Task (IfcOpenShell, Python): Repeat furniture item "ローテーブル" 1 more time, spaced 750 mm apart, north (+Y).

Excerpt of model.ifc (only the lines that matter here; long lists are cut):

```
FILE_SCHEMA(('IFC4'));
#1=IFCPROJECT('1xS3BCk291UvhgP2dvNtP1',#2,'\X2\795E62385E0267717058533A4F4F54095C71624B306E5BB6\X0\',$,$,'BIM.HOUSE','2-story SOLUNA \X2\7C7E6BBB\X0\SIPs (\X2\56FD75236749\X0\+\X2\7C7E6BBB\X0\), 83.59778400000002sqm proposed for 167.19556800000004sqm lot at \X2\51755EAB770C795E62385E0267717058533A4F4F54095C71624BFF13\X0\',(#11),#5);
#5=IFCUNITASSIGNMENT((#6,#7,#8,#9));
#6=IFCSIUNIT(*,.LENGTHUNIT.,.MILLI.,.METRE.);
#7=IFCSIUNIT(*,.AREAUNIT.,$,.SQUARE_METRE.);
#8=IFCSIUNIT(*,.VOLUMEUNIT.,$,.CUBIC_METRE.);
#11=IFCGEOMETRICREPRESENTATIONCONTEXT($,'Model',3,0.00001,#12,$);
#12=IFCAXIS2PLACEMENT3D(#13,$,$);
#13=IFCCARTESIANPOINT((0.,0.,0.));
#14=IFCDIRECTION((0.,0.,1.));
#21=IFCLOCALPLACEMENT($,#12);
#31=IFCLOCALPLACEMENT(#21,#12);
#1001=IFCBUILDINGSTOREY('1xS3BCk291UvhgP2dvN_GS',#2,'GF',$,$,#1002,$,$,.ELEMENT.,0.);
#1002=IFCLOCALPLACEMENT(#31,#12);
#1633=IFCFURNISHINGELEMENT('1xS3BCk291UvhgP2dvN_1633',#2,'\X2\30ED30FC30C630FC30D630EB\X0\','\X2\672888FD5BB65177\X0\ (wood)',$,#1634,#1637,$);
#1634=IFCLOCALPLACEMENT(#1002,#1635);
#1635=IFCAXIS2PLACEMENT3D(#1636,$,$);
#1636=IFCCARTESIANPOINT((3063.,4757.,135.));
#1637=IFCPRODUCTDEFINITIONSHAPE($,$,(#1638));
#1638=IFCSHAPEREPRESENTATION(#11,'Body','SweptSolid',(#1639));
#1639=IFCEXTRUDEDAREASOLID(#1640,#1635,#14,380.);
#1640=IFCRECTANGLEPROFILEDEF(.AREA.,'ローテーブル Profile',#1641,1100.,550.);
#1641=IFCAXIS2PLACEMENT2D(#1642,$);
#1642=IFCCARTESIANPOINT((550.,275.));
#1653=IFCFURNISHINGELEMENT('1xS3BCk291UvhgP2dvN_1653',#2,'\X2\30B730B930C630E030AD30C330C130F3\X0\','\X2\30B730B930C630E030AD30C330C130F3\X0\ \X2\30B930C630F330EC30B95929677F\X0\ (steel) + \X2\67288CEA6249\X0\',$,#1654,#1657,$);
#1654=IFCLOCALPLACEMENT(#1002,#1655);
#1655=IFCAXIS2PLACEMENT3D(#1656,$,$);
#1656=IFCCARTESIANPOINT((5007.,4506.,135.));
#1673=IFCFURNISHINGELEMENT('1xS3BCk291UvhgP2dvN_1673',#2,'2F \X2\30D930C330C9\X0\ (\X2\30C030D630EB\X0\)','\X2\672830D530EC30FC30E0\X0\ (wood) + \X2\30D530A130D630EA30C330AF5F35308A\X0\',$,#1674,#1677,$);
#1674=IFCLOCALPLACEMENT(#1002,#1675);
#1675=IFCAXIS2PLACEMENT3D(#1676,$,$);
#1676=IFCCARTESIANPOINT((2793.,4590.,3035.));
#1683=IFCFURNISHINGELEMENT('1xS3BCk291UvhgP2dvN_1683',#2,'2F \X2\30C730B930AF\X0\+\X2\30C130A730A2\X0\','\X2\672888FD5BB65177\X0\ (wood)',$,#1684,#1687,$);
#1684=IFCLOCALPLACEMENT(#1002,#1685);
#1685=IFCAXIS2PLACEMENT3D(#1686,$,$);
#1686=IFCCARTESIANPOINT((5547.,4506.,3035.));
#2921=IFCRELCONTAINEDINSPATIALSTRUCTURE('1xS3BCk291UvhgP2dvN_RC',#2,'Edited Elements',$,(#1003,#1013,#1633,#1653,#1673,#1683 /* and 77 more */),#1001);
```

```python
import numpy as np
import ifcopenshell
import ifcopenshell.api.geometry
import ifcopenshell.api.root
import ifcopenshell.util.element
import ifcopenshell.util.placement
import ifcopenshell.util.unit

model = ifcopenshell.open("model.ifc")
unit_scale = ifcopenshell.util.unit.calculate_unit_scale(model)


def reuse_history(source, copy):
    """copy_class also copies each property set's owner history, people and application; keep the originals."""
    for rel in copy.IsDefinedBy:
        if rel.is_a("IfcRelDefinesByProperties") and (history := rel.RelatingPropertyDefinition.OwnerHistory):
            rel.RelatingPropertyDefinition.OwnerHistory = source.OwnerHistory
            ifcopenshell.util.element.remove_deep2(model, history)


source = model.by_guid("1xS3BCk291UvhgP2dvN_1633")
base = ifcopenshell.util.placement.get_local_placement(source.ObjectPlacement)
step = np.array([0.0, 1.0, 0.0]) * 0.75 / unit_scale

for i in range(1, 2):
    copy = ifcopenshell.api.root.copy_class(model, product=source)
    copy.Representation = ifcopenshell.util.element.copy_deep(
        model, source.Representation, exclude=["IfcGeometricRepresentationContext", "IfcRepresentationMap"]
    )
    reuse_history(source, copy)
    matrix = base.copy()
    matrix[:3, 3] += i * step
    print("added at", matrix[:3, 3].round(3) + 0.0)
    ifcopenshell.api.geometry.edit_object_placement(model, product=copy, matrix=matrix, is_si=False)

model.write("model_edited.ifc")
```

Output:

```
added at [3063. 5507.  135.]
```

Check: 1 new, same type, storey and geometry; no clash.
